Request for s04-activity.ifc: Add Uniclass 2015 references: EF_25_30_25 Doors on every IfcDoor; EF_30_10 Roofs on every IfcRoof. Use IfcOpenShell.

First a look at what the model holds.

```python
import ifcopenshell

model = ifcopenshell.open("s04-activity.ifc")
print(model.schema)
print("classifications:", [c.Name for c in model.by_type("IfcClassification")])
for ifc_class in ("IfcDoor", "IfcRoof", "IfcStair", "IfcWall", "IfcWindow"):
    print(ifc_class, len(model.by_type(ifc_class)))
```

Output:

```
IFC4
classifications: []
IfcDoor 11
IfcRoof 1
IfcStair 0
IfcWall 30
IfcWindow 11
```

```python
import ifcopenshell
import ifcopenshell.api.classification

model = ifcopenshell.open("s04-activity.ifc")

system = ifcopenshell.api.classification.add_classification(model, classification="Uniclass 2015")

codes = {
    "IfcDoor": ("EF_25_30_25", "Doors"),
    "IfcRoof": ("EF_30_10", "Roofs"),
}
for ifc_class, (code, name) in codes.items():
    products = model.by_type(ifc_class)
    ifcopenshell.api.classification.add_reference(
        model, products=products, classification=system, identification=code, name=name
    )
    print(code, len(products))

model.write("s04-activity_rev.ifc")
```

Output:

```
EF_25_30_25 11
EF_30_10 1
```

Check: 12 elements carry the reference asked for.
